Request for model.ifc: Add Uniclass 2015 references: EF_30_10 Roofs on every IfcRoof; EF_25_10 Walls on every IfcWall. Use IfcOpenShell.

First a look at what the model holds.

```python
import ifcopenshell

model = ifcopenshell.open("model.ifc")
print(model.schema)
print("classifications:", [c.Name for c in model.by_type("IfcClassification")])
for ifc_class in ("IfcDoor", "IfcRoof", "IfcStair", "IfcWall", "IfcWindow"):
    print(ifc_class, len(model.by_type(ifc_class)))
```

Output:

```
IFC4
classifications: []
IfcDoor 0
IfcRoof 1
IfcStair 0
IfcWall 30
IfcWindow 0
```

```python
import ifcopenshell
import ifcopenshell.api.classification

model = ifcopenshell.open("model.ifc")

system = ifcopenshell.api.classification.add_classification(model, classification="Uniclass 2015")

codes = {
    "IfcRoof": ("EF_30_10", "Roofs"),
    "IfcWall": ("EF_25_10", "Walls"),
}
for ifc_class, (code, name) in codes.items():
    products = model.by_type(ifc_class)
    ifcopenshell.api.classification.add_reference(
        model, products=products, classification=system, identification=code, name=name
    )
    print(code, len(products))

model.write("model_edited.ifc")
```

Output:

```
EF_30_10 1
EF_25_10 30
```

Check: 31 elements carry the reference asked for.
